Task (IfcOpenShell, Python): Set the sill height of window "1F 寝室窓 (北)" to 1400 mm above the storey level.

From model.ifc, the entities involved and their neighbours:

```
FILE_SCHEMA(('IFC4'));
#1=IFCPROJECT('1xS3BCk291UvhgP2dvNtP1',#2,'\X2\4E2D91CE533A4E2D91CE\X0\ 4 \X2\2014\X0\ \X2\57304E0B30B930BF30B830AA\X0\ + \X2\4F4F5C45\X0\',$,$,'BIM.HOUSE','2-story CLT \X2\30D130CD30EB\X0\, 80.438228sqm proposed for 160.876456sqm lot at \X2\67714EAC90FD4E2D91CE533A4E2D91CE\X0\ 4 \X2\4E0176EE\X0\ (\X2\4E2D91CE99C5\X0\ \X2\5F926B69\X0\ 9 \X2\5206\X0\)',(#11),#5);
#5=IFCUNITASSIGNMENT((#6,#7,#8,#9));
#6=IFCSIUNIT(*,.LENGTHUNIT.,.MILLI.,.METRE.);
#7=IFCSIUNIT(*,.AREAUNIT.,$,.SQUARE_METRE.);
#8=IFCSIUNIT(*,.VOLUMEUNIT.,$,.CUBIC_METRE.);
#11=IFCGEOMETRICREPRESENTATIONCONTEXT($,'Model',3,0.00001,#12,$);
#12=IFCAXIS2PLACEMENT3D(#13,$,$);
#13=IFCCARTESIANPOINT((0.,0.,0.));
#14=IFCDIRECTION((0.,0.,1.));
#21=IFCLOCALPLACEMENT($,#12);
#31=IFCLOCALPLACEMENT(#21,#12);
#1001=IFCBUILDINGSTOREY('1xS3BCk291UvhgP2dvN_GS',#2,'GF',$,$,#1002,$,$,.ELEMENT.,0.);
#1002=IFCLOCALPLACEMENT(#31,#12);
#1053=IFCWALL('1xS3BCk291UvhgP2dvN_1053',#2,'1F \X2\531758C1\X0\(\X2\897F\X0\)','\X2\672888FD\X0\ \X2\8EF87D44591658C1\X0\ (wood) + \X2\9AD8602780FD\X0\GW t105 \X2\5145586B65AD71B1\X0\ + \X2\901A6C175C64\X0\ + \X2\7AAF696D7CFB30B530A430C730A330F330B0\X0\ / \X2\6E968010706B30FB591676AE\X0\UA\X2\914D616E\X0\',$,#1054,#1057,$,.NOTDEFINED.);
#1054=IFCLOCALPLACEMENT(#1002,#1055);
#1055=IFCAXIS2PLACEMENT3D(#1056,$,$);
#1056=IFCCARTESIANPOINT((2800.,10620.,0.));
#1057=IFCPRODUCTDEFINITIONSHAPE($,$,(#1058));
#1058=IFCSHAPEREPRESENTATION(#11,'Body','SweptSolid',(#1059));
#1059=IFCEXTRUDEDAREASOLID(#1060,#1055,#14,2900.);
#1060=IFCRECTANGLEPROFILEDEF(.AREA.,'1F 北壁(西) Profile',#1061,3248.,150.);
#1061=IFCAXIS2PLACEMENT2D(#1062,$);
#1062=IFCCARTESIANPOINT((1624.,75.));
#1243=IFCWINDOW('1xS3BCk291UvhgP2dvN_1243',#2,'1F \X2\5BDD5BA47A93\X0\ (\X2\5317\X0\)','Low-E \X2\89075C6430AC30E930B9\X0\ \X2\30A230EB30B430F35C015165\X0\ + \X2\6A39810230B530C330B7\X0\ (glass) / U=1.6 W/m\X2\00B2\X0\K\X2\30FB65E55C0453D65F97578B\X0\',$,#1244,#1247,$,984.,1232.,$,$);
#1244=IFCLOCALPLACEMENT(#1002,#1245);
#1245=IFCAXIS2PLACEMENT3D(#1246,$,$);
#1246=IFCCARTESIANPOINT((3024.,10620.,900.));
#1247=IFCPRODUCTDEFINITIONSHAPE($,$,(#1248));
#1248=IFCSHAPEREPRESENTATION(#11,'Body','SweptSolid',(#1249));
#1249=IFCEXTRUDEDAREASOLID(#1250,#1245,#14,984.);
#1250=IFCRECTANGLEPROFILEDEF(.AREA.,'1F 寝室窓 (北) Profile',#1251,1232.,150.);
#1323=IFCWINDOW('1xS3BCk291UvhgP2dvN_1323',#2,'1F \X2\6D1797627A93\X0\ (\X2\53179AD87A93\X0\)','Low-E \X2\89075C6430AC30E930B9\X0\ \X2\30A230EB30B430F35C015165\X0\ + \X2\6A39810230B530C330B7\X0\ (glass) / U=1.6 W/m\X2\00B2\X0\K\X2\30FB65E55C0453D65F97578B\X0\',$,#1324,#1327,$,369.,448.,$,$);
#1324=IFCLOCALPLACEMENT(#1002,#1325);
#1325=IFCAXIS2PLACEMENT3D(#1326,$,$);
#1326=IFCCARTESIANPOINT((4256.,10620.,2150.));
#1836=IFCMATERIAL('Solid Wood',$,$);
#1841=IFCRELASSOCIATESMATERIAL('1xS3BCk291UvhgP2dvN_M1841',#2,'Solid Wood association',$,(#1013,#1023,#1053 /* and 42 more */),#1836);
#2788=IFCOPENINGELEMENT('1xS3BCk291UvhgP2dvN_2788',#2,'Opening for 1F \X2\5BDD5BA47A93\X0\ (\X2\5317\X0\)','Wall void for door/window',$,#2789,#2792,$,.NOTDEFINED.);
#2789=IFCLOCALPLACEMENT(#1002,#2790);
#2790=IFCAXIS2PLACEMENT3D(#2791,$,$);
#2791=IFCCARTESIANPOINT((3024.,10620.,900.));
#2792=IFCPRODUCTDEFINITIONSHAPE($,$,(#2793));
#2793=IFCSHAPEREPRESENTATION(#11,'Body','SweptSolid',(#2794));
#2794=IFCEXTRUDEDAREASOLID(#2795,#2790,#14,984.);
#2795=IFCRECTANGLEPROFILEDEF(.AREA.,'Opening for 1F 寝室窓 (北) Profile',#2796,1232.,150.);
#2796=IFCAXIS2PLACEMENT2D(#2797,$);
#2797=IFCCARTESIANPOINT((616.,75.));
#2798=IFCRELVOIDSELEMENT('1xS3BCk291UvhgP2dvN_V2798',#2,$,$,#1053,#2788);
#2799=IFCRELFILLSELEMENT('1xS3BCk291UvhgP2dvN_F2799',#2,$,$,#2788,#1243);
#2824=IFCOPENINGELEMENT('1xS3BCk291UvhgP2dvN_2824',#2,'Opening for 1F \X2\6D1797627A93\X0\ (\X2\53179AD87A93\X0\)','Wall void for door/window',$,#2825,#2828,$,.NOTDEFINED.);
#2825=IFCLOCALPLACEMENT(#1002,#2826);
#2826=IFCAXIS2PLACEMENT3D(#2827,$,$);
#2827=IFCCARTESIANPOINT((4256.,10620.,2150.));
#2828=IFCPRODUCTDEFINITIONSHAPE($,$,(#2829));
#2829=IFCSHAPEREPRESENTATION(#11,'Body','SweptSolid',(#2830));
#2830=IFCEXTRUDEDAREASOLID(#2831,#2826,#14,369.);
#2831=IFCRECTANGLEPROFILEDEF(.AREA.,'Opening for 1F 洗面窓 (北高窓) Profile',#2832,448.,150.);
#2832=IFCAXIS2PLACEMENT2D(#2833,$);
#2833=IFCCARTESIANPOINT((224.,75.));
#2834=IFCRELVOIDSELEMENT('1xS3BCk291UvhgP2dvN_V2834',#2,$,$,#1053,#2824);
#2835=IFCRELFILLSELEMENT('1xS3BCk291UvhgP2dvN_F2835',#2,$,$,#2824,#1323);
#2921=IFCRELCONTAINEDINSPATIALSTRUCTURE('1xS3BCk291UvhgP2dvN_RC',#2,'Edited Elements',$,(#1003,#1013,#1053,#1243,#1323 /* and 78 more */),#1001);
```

```python
import numpy as np
import ifcopenshell
import ifcopenshell.api.geometry
import ifcopenshell.geom
import ifcopenshell.util.element
import ifcopenshell.util.placement
import ifcopenshell.util.shape
import ifcopenshell.util.unit

model = ifcopenshell.open("model.ifc")
unit_scale = ifcopenshell.util.unit.calculate_unit_scale(model)

window = model.by_guid("1xS3BCk291UvhgP2dvN_1243")
opening = window.FillsVoids[0].RelatingOpeningElement
storey = ifcopenshell.util.element.get_container(window, ifc_class="IfcBuildingStorey")
level = ifcopenshell.util.placement.get_local_placement(storey.ObjectPlacement)[2, 3]

# The opening's origin need not be at the sill, so measure its lowest point.
shape = ifcopenshell.geom.create_shape(ifcopenshell.geom.settings(), opening)
bottom = ifcopenshell.util.shape.get_shape_bottom_elevation(shape, shape.geometry) / unit_scale
dz = level + 1400.0 - bottom

shift = np.array([0.0, 0.0, dz])
# The window is not placed relative to its opening, so move both.
for product in (opening, window):
    matrix = ifcopenshell.util.placement.get_local_placement(product.ObjectPlacement)
    matrix[:3, 3] += shift
    ifcopenshell.api.geometry.edit_object_placement(model, product=product, matrix=matrix, is_si=False)

print(f"moved by {dz * unit_scale:+.3f} m")

model.write("model_edited.ifc")
```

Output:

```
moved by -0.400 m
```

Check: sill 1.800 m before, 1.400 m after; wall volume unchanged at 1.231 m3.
